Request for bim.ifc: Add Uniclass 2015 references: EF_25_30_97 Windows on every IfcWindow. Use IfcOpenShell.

First a look at what the model holds.

```python
import ifcopenshell

model = ifcopenshell.open("bim.ifc")
print(model.schema)
print("classifications:", [c.Name for c in model.by_type("IfcClassification")])
for ifc_class in ("IfcDoor", "IfcRoof", "IfcStair", "IfcWall", "IfcWindow"):
    print(ifc_class, len(model.by_type(ifc_class)))
```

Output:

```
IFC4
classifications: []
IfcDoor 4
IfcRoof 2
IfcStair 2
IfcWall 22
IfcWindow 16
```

```python
import ifcopenshell
import ifcopenshell.api.classification

model = ifcopenshell.open("bim.ifc")

system = ifcopenshell.api.classification.add_classification(model, classification="Uniclass 2015")

codes = {
    "IfcWindow": ("EF_25_30_97", "Windows"),
}
for ifc_class, (code, name) in codes.items():
    products = model.by_type(ifc_class)
    ifcopenshell.api.classification.add_reference(
        model, products=products, classification=system, identification=code, name=name
    )
    print(code, len(products))

model.write("bim_rev.ifc")
```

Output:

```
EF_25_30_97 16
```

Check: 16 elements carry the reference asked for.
